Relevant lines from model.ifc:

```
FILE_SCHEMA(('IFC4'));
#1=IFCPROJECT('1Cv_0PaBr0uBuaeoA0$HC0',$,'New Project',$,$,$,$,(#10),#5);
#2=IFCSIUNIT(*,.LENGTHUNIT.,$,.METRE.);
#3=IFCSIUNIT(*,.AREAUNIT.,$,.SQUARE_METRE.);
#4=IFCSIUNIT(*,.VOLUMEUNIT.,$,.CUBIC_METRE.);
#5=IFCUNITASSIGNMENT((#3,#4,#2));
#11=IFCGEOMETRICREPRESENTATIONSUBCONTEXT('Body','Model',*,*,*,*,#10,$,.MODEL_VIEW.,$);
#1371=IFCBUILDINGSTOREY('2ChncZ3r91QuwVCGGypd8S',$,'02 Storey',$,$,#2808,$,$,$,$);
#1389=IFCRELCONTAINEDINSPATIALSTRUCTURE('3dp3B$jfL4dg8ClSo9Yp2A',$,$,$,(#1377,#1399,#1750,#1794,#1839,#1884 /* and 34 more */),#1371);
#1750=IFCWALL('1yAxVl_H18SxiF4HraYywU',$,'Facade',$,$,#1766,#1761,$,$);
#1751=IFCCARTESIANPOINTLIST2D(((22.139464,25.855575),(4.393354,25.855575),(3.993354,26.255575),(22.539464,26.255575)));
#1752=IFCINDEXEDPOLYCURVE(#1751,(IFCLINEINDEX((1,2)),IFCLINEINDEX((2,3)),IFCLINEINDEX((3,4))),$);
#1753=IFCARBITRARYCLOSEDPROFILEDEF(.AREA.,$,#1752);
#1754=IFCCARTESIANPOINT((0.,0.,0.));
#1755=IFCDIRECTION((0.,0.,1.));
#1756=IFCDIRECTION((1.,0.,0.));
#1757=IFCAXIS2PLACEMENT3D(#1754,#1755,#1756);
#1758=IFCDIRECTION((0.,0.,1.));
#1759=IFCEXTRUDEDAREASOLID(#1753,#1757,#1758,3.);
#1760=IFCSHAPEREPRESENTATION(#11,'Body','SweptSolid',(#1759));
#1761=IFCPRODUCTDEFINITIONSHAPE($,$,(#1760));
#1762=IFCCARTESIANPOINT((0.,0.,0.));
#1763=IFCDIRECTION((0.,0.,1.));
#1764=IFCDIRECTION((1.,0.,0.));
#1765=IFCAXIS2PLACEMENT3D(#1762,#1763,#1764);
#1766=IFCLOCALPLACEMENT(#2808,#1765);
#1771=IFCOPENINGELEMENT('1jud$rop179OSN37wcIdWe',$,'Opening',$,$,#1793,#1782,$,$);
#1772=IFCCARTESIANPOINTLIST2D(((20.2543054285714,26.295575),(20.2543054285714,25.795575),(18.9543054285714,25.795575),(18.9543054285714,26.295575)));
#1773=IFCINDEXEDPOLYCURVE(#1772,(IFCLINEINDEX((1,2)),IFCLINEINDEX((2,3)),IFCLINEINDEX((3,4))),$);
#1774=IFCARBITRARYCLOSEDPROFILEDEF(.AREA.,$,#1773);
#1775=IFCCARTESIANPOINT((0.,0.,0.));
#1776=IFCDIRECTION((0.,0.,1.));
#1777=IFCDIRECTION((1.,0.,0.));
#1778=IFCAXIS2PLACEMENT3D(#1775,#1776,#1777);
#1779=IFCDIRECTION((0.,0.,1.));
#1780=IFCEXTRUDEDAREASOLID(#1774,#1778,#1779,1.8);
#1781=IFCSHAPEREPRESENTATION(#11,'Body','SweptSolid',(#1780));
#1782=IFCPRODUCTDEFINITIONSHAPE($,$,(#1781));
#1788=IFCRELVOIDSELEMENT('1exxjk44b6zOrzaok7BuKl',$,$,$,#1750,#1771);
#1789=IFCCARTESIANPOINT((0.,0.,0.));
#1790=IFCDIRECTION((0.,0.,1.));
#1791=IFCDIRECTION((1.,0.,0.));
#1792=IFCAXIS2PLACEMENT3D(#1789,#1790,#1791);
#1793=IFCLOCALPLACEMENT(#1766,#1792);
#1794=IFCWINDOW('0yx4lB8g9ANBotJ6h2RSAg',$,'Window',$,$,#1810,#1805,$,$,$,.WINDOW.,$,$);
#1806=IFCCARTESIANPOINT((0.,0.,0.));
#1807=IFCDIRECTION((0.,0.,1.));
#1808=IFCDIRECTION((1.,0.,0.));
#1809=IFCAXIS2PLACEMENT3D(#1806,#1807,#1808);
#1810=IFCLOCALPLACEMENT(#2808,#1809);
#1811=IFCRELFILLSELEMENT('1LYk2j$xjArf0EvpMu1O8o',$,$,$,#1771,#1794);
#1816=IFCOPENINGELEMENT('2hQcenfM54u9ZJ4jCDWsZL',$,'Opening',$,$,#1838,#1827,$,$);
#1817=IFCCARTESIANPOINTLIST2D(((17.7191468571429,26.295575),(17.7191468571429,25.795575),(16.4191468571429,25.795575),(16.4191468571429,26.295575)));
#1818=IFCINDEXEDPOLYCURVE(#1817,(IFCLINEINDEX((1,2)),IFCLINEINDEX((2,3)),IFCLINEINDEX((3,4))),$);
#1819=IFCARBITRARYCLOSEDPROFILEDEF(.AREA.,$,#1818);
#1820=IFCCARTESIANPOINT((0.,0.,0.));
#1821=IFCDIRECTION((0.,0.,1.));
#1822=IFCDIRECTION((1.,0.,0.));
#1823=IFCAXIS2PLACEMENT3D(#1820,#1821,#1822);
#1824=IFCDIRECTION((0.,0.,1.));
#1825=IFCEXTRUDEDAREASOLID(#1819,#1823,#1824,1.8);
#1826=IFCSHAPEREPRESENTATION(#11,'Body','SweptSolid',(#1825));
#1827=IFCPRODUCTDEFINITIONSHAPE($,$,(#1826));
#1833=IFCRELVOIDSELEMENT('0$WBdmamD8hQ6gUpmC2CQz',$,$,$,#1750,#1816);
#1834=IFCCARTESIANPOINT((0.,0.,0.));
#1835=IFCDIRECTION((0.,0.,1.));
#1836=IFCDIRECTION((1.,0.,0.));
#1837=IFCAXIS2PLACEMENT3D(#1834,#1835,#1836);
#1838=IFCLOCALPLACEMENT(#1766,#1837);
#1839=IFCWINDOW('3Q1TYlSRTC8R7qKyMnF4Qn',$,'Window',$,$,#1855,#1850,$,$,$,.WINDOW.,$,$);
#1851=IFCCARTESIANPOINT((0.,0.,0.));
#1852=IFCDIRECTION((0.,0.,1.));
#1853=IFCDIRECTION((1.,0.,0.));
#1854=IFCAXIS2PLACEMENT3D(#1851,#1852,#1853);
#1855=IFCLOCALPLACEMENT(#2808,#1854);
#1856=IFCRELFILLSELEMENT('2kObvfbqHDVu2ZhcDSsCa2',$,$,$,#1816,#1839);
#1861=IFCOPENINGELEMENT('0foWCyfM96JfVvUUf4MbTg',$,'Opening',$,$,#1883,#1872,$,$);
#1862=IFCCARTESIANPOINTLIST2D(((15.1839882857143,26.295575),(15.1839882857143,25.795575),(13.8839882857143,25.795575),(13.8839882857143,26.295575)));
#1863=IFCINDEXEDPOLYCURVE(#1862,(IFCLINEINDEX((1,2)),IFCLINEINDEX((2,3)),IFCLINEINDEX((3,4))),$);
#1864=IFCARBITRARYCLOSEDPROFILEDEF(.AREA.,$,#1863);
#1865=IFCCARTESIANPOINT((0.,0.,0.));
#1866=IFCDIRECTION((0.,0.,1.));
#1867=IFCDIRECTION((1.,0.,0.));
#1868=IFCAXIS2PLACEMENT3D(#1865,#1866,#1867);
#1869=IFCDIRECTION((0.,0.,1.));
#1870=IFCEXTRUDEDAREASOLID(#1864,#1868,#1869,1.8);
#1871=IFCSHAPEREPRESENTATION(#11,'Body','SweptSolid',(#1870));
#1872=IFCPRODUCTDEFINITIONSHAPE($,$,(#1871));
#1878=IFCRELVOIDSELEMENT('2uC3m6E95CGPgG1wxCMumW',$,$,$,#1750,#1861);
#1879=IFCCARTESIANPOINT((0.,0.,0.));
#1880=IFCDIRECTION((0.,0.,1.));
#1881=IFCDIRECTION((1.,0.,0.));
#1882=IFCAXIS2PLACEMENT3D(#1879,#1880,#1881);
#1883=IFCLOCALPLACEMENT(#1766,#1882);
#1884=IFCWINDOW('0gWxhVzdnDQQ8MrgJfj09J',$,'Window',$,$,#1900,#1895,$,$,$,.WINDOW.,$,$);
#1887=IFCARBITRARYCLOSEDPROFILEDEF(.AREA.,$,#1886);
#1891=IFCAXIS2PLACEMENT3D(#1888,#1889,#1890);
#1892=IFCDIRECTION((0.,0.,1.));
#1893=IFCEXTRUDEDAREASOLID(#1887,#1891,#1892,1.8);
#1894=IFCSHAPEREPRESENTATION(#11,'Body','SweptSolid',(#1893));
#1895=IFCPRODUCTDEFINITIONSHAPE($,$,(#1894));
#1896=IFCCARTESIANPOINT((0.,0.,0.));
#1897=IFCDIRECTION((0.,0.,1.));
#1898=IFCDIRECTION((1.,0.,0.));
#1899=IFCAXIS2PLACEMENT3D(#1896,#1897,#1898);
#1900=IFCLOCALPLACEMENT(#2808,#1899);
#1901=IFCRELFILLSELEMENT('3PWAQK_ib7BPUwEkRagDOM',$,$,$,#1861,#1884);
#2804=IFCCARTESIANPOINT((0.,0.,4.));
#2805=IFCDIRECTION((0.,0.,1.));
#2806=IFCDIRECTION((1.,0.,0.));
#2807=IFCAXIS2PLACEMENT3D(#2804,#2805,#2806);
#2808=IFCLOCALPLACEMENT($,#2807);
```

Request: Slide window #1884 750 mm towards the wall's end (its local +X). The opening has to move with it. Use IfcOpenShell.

```python
import ifcopenshell
import ifcopenshell.api.geometry
import ifcopenshell.util.placement
import ifcopenshell.util.unit

model = ifcopenshell.open("model.ifc")
unit_scale = ifcopenshell.util.unit.calculate_unit_scale(model)

window = model.by_id(1884)
opening = window.FillsVoids[0].RelatingOpeningElement
wall = opening.VoidsElements[0].RelatingBuildingElement

wall_matrix = ifcopenshell.util.placement.get_local_placement(wall.ObjectPlacement)
shift = wall_matrix[:3, 0] * 0.75 / unit_scale
before = ifcopenshell.util.placement.get_local_placement(window.ObjectPlacement)[:3, 3].copy()

# The window is not placed relative to its opening, so move both.
for product in (opening, window):
    matrix = ifcopenshell.util.placement.get_local_placement(product.ObjectPlacement)
    matrix[:3, 3] += shift
    ifcopenshell.api.geometry.edit_object_placement(model, product=product, matrix=matrix, is_si=False)

after = ifcopenshell.util.placement.get_local_placement(window.ObjectPlacement)[:3, 3]
print("window moved by", (after - before).round(3) + 0.0)

model.write("model-out.ifc")
```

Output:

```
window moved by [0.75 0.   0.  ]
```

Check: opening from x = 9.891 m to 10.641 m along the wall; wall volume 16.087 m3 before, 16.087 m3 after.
